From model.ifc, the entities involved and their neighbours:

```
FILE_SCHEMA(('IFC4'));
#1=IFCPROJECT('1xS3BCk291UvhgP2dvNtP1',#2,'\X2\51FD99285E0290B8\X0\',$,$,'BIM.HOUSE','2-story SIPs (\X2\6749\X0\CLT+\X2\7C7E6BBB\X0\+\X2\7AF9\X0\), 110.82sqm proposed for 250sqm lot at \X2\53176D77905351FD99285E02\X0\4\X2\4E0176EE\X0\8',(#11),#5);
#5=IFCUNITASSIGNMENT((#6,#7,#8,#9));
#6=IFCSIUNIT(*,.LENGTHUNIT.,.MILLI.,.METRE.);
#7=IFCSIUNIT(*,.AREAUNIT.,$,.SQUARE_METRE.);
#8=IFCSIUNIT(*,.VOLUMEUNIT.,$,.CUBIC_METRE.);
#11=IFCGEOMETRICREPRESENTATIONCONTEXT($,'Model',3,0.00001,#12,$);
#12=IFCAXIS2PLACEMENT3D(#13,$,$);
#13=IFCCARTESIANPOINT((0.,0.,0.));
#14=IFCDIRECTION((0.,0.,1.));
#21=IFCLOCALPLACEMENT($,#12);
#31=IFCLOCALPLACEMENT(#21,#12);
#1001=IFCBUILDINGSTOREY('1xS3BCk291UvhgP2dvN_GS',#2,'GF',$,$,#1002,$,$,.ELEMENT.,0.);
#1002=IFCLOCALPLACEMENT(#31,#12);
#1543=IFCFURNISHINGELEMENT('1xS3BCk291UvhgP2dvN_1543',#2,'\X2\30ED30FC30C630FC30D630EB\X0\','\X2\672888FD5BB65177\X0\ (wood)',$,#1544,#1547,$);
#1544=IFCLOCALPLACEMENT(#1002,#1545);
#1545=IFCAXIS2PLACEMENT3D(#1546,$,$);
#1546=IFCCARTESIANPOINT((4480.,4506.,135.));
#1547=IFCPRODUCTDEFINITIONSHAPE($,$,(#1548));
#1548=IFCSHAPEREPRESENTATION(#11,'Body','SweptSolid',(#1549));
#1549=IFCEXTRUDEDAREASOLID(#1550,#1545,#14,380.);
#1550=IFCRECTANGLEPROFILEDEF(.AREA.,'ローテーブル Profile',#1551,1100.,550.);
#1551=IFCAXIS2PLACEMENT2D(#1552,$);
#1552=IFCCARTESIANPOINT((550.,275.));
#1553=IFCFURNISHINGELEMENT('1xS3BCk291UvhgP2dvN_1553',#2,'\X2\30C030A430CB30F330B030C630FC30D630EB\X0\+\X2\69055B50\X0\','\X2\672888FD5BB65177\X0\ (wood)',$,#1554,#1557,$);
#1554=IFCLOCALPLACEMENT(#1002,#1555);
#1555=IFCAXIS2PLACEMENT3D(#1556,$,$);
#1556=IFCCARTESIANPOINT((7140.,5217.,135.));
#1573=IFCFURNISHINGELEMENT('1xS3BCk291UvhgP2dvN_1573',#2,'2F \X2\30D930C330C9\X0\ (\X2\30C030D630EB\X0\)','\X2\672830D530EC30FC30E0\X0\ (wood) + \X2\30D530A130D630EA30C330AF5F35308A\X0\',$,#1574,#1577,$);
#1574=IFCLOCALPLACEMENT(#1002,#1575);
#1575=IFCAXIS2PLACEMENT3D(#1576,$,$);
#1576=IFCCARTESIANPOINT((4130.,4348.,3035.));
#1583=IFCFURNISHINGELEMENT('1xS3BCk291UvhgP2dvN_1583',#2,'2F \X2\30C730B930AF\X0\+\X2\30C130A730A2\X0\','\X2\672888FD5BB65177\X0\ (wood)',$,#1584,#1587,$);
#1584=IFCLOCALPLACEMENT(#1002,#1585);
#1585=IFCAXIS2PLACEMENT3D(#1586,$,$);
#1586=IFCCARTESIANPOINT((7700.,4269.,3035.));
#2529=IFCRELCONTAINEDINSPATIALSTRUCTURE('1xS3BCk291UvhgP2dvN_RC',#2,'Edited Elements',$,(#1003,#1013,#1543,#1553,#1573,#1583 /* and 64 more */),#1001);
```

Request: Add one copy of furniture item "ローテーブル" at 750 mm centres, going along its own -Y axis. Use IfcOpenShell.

```python
import ifcopenshell
import ifcopenshell.api.geometry
import ifcopenshell.api.root
import ifcopenshell.util.element
import ifcopenshell.util.placement
import ifcopenshell.util.unit

model = ifcopenshell.open("model.ifc")
unit_scale = ifcopenshell.util.unit.calculate_unit_scale(model)


def reuse_history(source, copy):
    """copy_class also copies each property set's owner history, people and application; keep the originals."""
    for rel in copy.IsDefinedBy:
        if rel.is_a("IfcRelDefinesByProperties") and (history := rel.RelatingPropertyDefinition.OwnerHistory):
            rel.RelatingPropertyDefinition.OwnerHistory = source.OwnerHistory
            ifcopenshell.util.element.remove_deep2(model, history)


source = model.by_guid("1xS3BCk291UvhgP2dvN_1543")
base = ifcopenshell.util.placement.get_local_placement(source.ObjectPlacement)
step = -base[:3, 1] * 0.75 / unit_scale

for i in range(1, 2):
    copy = ifcopenshell.api.root.copy_class(model, product=source)
    copy.Representation = ifcopenshell.util.element.copy_deep(
        model, source.Representation, exclude=["IfcGeometricRepresentationContext", "IfcRepresentationMap"]
    )
    reuse_history(source, copy)
    matrix = base.copy()
    matrix[:3, 3] += i * step
    print("added at", matrix[:3, 3].round(3) + 0.0)
    ifcopenshell.api.geometry.edit_object_placement(model, product=copy, matrix=matrix, is_si=False)

model.write("model_v2.ifc")
```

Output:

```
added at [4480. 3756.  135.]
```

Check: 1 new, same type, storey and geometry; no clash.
